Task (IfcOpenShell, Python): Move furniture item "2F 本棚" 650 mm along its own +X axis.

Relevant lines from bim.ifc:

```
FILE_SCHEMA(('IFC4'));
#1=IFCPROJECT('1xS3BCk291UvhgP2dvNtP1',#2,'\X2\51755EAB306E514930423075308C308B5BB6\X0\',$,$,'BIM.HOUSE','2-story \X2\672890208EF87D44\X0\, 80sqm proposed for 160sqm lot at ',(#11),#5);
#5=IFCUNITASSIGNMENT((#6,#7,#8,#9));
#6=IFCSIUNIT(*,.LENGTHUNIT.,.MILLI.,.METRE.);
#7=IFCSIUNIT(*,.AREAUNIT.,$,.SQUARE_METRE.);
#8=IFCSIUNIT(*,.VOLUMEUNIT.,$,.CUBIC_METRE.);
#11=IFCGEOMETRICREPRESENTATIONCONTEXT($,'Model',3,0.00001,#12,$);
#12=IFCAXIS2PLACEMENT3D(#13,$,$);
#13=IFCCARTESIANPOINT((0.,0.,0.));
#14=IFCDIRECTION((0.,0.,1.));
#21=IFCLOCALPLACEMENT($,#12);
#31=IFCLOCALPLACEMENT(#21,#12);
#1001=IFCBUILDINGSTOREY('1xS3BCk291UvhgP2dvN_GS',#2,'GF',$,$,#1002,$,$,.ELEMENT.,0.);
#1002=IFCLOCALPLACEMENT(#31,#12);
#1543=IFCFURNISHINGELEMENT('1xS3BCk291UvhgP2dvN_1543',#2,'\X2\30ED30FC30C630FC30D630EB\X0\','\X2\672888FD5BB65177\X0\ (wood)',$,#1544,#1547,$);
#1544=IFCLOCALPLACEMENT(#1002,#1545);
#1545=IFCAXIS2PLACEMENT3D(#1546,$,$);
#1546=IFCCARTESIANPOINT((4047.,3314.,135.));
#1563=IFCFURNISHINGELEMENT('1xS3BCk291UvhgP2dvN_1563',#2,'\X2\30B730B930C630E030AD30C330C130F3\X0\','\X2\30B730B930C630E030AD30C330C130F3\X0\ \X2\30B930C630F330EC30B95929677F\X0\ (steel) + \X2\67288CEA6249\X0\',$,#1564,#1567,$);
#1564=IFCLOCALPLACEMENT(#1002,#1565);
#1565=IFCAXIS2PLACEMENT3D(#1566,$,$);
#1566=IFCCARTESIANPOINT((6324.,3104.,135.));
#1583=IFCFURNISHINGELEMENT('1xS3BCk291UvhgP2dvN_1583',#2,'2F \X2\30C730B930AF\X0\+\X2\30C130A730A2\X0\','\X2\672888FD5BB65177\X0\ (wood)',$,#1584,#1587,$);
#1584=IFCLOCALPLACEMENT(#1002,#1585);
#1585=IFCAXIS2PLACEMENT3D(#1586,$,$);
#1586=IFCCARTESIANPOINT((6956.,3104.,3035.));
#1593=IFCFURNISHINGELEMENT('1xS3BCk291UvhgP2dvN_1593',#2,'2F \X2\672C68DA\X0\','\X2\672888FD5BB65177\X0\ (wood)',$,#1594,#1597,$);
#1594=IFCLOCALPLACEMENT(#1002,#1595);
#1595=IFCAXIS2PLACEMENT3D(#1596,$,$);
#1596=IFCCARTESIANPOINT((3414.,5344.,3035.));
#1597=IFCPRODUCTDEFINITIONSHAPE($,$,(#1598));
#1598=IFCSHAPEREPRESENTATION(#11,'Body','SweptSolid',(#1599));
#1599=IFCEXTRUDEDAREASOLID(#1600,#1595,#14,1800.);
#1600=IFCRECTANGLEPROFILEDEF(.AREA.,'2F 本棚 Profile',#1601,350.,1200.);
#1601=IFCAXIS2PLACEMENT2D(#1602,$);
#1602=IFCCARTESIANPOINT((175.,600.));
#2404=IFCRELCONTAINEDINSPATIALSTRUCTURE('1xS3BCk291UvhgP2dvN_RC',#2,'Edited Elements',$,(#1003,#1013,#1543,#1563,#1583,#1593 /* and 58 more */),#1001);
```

```python
import ifcopenshell
import ifcopenshell.api.geometry
import ifcopenshell.util.placement

model = ifcopenshell.open("bim.ifc")

item = model.by_guid("1xS3BCk291UvhgP2dvN_1593")
matrix = ifcopenshell.util.placement.get_local_placement(item.ObjectPlacement)
matrix[:3, 3] += matrix[:3, 0] * 650.0
ifcopenshell.api.geometry.edit_object_placement(model, product=item, matrix=matrix, is_si=False)

print(ifcopenshell.util.placement.get_local_placement(item.ObjectPlacement).round(3) + 0.0)

model.write("bim-out.ifc")
```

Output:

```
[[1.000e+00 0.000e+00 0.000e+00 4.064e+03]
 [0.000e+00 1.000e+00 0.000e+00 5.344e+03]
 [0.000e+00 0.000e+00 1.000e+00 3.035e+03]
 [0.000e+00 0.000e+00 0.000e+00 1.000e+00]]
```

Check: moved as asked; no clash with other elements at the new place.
